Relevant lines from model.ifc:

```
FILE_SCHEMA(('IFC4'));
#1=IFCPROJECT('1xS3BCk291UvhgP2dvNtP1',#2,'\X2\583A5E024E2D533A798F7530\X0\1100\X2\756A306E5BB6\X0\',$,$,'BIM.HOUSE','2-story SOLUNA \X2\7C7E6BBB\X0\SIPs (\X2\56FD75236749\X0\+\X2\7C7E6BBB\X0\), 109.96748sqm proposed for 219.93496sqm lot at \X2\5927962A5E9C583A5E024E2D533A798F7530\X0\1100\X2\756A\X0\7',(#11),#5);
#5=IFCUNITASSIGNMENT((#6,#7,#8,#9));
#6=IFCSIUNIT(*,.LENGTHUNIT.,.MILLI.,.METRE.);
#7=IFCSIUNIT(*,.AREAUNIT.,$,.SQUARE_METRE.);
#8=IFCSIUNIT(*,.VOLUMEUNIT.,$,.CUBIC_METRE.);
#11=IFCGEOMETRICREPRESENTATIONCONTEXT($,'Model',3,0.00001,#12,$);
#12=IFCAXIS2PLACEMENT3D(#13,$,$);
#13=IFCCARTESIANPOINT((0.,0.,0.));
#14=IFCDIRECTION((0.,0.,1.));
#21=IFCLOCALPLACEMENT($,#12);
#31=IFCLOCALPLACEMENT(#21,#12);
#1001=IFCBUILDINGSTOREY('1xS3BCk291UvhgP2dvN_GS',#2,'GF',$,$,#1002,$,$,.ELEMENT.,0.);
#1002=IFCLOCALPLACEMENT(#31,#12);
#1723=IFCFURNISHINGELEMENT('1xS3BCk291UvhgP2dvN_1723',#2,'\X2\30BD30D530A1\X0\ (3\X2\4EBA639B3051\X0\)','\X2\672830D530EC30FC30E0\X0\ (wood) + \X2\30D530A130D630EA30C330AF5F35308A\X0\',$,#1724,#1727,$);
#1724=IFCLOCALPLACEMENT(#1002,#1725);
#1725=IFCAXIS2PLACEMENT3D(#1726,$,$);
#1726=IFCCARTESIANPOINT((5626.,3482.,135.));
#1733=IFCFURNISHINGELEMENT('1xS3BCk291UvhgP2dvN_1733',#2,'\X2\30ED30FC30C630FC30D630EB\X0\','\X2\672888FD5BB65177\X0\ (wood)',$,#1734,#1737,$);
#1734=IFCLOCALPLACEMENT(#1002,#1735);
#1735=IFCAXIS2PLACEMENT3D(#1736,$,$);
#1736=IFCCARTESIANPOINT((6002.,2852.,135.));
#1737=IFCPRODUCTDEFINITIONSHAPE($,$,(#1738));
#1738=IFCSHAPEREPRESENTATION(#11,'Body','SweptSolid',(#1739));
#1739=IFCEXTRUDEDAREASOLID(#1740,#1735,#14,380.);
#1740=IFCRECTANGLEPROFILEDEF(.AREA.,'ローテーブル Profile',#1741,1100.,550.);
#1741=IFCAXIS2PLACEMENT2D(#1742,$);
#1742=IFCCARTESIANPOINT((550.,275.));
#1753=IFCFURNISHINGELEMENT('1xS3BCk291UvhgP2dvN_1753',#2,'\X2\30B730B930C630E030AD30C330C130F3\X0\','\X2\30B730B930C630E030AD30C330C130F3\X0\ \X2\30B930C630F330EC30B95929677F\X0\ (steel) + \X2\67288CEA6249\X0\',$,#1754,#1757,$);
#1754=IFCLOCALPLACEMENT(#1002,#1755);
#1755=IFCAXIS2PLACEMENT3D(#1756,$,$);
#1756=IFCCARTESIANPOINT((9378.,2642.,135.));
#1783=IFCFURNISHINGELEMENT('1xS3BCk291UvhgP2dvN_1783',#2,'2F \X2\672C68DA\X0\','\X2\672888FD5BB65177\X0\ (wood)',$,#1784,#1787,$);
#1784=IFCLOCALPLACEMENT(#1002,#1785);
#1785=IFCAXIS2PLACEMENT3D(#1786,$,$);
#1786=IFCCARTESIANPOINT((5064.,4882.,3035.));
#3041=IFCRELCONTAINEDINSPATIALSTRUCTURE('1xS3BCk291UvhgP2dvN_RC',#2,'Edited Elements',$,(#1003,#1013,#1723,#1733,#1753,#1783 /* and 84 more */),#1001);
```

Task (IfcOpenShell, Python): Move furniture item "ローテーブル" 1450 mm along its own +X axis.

```python
import ifcopenshell
import ifcopenshell.api.geometry
import ifcopenshell.util.placement

model = ifcopenshell.open("model.ifc")

item = model.by_guid("1xS3BCk291UvhgP2dvN_1733")
matrix = ifcopenshell.util.placement.get_local_placement(item.ObjectPlacement)
matrix[:3, 3] += matrix[:3, 0] * 1450.0
ifcopenshell.api.geometry.edit_object_placement(model, product=item, matrix=matrix, is_si=False)

print(ifcopenshell.util.placement.get_local_placement(item.ObjectPlacement).round(3) + 0.0)

model.write("model_edited.ifc")
```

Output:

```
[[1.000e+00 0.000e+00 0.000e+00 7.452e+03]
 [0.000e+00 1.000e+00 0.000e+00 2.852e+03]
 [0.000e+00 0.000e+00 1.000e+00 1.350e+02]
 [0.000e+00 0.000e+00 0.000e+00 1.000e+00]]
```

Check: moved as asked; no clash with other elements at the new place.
